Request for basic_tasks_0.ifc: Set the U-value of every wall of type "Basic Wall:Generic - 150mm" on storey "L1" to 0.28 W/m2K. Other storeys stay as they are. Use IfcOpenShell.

First a look at what the model holds.

```python
import ifcopenshell
import ifcopenshell.util.element

model = ifcopenshell.open("basic_tasks_0.ifc")
print(model.schema)
storey = next(s for s in model.by_type("IfcBuildingStorey") if s.Name == "L1")
walls = [e for e in ifcopenshell.util.element.get_decomposition(storey) if e.is_a("IfcWall")]
seen = {}
for e in walls:
    element_type = ifcopenshell.util.element.get_type(e)
    key = (element_type.Name if element_type != e and element_type else None, ifcopenshell.util.element.get_pset(e, "Pset_WallCommon", "ThermalTransmittance"))
    seen[key] = seen.get(key, 0) + 1
for (name, value), count in sorted(seen.items(), key=str):
    print(count, "x", name, "|", value)
```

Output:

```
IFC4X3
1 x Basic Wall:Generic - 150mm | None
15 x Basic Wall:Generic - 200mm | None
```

```python
import ifcopenshell
import ifcopenshell.api.pset
import ifcopenshell.util.element

model = ifcopenshell.open("basic_tasks_0.ifc")

storey = next(s for s in model.by_type("IfcBuildingStorey") if s.Name == "L1")
walls = [e for e in ifcopenshell.util.element.get_decomposition(storey) if e.is_a("IfcWall")]

count = 0
for e in walls:
    element_type = ifcopenshell.util.element.get_type(e)
    if element_type in (None, e) or element_type.Name != "Basic Wall:Generic - 150mm":
        continue
    # add_pset returns the element's existing set when there is one.
    pset = ifcopenshell.api.pset.add_pset(model, product=e, name="Pset_WallCommon")
    ifcopenshell.api.pset.edit_pset(model, pset=pset, properties={"ThermalTransmittance": 0.28})
    count += 1

print(count, "walls updated")

model.write("basic_tasks_0_updated.ifc")
```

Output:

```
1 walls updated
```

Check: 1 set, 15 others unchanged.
